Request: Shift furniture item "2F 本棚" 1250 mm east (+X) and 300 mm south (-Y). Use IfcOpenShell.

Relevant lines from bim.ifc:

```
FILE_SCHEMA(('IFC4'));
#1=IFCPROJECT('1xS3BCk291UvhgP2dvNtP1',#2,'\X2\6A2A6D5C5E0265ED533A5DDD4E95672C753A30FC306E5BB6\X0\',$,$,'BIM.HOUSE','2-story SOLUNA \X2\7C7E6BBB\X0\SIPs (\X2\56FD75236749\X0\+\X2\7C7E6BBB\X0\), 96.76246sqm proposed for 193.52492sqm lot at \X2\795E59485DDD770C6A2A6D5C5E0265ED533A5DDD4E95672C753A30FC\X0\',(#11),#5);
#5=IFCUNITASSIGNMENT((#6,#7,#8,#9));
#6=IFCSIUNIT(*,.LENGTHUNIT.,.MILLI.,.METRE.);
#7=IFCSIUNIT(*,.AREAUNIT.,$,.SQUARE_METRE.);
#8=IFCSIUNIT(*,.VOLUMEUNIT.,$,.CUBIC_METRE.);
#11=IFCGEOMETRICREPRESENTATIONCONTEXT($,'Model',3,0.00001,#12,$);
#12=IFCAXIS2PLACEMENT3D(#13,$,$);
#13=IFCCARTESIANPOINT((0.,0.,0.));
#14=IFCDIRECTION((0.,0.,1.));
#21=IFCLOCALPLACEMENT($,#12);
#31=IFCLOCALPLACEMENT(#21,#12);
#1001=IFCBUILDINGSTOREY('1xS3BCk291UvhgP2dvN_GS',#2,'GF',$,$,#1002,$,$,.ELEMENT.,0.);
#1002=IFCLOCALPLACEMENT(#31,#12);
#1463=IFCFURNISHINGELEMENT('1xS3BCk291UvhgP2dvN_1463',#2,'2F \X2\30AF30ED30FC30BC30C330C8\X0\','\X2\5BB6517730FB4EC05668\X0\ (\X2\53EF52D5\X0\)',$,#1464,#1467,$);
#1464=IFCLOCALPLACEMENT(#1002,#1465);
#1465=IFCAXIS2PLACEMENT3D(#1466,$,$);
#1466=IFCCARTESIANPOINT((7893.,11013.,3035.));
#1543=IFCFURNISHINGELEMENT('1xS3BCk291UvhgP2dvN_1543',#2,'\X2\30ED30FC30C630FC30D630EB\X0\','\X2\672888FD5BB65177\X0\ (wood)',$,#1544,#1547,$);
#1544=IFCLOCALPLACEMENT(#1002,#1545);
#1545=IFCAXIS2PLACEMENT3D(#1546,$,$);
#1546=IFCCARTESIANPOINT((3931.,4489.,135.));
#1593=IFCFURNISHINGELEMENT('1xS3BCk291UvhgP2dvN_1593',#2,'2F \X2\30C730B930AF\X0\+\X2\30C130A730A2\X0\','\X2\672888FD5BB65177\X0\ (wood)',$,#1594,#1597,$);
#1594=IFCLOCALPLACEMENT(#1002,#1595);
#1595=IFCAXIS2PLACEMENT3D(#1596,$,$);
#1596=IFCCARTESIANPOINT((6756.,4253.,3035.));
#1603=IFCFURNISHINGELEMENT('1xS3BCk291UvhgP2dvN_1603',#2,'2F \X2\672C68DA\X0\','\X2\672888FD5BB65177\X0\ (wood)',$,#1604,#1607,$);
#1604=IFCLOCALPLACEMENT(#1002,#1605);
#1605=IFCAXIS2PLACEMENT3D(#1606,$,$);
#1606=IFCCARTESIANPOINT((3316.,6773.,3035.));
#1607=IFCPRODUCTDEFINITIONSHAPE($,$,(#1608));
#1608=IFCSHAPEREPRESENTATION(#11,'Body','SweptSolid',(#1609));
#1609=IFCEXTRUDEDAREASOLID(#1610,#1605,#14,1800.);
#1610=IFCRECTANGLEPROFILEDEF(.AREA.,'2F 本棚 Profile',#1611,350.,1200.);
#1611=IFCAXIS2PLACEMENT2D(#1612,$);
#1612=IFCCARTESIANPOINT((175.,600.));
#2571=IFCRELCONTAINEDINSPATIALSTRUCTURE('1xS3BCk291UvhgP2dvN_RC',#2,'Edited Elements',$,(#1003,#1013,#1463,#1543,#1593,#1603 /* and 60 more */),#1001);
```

```python
import ifcopenshell
import ifcopenshell.api.geometry
import ifcopenshell.util.placement
import ifcopenshell.util.unit

model = ifcopenshell.open("bim.ifc")
unit_scale = ifcopenshell.util.unit.calculate_unit_scale(model)

item = model.by_guid("1xS3BCk291UvhgP2dvN_1603")
matrix = ifcopenshell.util.placement.get_local_placement(item.ObjectPlacement)
matrix[0, 3] += 1.25 / unit_scale
matrix[1, 3] -= 0.3 / unit_scale
ifcopenshell.api.geometry.edit_object_placement(model, product=item, matrix=matrix, is_si=False)

print(ifcopenshell.util.placement.get_local_placement(item.ObjectPlacement).round(3) + 0.0)

model.write("bim_v2.ifc")
```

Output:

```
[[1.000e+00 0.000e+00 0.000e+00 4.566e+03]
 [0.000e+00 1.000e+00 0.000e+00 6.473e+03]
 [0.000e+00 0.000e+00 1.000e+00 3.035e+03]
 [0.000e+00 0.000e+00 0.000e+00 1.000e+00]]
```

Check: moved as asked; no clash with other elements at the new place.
